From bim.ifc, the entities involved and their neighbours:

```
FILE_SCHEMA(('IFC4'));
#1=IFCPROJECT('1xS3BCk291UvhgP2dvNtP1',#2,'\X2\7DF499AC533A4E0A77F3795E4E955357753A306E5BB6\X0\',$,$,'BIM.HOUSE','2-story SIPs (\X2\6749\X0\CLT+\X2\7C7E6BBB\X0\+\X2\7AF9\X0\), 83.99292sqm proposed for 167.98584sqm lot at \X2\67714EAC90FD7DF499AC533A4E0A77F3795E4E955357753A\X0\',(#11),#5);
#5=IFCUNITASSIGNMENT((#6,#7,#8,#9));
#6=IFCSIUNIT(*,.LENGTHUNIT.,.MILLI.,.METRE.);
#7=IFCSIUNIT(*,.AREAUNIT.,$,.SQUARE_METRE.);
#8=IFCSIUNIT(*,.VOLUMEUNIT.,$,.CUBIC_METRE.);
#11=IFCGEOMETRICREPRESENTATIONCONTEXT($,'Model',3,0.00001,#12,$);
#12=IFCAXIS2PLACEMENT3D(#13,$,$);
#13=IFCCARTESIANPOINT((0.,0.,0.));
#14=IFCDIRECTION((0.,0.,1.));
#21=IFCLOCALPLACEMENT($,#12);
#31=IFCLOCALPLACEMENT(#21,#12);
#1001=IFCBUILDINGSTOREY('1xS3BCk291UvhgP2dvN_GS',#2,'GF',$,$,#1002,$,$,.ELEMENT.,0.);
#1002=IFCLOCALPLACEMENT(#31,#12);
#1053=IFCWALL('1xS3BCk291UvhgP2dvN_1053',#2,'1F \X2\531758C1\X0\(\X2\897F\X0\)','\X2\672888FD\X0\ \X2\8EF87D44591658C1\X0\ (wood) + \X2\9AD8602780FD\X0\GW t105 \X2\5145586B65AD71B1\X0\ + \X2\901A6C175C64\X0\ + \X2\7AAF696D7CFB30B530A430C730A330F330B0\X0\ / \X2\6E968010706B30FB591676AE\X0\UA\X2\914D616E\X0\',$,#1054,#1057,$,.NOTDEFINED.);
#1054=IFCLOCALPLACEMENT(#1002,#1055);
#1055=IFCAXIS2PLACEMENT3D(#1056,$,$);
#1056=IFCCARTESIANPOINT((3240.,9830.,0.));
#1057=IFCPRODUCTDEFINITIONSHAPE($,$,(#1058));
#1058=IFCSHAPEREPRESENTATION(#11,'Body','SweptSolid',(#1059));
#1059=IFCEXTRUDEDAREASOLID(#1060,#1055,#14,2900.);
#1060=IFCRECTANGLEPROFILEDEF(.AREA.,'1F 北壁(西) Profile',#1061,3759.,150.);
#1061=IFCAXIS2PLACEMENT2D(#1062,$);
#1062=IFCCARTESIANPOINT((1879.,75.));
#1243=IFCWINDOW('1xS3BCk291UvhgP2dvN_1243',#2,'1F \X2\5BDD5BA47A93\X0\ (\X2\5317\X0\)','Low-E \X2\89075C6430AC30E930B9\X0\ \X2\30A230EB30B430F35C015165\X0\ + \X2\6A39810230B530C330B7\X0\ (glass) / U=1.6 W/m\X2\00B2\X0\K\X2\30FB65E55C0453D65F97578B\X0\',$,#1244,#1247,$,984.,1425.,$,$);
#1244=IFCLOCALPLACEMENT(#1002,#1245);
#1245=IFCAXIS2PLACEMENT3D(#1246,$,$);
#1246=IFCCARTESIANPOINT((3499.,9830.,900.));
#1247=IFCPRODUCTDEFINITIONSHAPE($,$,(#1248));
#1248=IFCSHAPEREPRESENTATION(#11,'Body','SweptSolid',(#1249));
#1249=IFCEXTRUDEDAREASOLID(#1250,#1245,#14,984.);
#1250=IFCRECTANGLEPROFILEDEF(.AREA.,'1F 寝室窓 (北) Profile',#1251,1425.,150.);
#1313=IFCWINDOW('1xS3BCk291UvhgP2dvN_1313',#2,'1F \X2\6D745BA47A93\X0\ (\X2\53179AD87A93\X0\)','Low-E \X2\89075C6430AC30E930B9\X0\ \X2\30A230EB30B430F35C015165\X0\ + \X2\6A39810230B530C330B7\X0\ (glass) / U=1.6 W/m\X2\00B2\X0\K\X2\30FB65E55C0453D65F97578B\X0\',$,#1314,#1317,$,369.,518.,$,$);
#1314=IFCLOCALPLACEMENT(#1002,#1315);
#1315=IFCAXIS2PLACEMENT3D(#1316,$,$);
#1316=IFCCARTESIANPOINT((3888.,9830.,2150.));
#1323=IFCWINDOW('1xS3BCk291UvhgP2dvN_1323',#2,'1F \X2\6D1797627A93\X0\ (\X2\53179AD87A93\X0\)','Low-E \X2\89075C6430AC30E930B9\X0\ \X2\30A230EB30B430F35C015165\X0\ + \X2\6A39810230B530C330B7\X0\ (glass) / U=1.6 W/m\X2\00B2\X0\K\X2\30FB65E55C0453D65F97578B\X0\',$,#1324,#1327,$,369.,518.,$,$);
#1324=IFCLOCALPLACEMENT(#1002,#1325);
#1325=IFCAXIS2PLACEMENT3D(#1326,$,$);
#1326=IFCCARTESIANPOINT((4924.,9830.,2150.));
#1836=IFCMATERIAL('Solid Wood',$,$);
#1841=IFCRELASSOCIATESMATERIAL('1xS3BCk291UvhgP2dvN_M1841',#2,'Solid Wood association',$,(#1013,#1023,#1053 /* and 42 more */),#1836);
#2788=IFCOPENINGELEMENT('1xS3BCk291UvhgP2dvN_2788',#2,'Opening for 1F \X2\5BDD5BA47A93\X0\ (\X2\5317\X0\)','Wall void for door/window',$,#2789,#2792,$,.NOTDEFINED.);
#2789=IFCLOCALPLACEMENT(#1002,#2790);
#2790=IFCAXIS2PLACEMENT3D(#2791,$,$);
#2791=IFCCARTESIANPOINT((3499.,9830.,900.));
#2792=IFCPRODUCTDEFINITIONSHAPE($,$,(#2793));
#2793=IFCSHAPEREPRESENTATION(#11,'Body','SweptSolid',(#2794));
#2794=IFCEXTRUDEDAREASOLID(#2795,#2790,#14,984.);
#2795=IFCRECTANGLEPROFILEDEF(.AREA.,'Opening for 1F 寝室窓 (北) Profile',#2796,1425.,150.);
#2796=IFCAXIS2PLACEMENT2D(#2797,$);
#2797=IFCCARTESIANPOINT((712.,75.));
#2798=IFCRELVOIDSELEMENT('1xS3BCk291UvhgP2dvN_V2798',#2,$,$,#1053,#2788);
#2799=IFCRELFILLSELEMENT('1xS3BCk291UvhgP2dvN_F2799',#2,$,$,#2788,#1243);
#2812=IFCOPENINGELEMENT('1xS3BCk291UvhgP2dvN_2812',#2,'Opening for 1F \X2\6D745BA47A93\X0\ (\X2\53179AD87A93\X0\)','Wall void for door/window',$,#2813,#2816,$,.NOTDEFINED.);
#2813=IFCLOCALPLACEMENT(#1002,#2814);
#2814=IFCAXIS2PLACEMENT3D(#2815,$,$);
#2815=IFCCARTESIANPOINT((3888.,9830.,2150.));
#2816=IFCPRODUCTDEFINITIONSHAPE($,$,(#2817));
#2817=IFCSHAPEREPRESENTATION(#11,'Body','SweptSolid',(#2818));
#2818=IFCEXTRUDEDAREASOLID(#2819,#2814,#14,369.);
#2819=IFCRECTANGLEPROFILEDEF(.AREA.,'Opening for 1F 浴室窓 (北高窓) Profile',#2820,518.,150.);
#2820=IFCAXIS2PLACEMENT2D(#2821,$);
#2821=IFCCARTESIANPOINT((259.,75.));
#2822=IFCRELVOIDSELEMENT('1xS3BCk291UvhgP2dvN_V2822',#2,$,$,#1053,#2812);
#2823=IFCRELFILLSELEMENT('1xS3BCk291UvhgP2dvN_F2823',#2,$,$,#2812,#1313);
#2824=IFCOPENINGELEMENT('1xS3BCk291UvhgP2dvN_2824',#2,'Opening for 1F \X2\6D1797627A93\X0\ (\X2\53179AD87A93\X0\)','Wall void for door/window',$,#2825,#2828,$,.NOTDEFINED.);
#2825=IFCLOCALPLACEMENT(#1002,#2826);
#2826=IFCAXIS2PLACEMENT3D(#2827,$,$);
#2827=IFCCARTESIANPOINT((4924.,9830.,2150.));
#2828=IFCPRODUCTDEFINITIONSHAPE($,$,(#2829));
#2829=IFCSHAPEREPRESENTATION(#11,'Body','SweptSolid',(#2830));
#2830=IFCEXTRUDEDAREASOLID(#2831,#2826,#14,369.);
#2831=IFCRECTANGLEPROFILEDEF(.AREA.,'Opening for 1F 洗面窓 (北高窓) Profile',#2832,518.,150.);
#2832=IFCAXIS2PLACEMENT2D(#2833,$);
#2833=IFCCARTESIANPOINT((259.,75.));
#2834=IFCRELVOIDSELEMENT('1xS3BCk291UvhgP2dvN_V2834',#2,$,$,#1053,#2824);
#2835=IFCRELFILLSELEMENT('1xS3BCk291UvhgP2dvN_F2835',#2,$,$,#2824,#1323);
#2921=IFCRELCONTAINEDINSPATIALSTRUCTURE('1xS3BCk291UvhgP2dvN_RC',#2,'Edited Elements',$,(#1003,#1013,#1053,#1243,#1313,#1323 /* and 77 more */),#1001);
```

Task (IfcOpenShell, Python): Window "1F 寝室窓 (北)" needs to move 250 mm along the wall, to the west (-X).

```python
import ifcopenshell
import ifcopenshell.api.geometry
import ifcopenshell.util.placement

model = ifcopenshell.open("bim.ifc")

window = model.by_guid("1xS3BCk291UvhgP2dvN_1243")
opening = window.FillsVoids[0].RelatingOpeningElement
wall = opening.VoidsElements[0].RelatingBuildingElement

wall_matrix = ifcopenshell.util.placement.get_local_placement(wall.ObjectPlacement)
shift = wall_matrix[:3, 0] * -250.0
before = ifcopenshell.util.placement.get_local_placement(window.ObjectPlacement)[:3, 3].copy()

# The window is not placed relative to its opening, so move both.
for product in (opening, window):
    matrix = ifcopenshell.util.placement.get_local_placement(product.ObjectPlacement)
    matrix[:3, 3] += shift
    ifcopenshell.api.geometry.edit_object_placement(model, product=product, matrix=matrix, is_si=False)

after = ifcopenshell.util.placement.get_local_placement(window.ObjectPlacement)[:3, 3]
print("window moved by", (after - before).round(3) + 0.0)

model.write("bim_edited.ifc")
```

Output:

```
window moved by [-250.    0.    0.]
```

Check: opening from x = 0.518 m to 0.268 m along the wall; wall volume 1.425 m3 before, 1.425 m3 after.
